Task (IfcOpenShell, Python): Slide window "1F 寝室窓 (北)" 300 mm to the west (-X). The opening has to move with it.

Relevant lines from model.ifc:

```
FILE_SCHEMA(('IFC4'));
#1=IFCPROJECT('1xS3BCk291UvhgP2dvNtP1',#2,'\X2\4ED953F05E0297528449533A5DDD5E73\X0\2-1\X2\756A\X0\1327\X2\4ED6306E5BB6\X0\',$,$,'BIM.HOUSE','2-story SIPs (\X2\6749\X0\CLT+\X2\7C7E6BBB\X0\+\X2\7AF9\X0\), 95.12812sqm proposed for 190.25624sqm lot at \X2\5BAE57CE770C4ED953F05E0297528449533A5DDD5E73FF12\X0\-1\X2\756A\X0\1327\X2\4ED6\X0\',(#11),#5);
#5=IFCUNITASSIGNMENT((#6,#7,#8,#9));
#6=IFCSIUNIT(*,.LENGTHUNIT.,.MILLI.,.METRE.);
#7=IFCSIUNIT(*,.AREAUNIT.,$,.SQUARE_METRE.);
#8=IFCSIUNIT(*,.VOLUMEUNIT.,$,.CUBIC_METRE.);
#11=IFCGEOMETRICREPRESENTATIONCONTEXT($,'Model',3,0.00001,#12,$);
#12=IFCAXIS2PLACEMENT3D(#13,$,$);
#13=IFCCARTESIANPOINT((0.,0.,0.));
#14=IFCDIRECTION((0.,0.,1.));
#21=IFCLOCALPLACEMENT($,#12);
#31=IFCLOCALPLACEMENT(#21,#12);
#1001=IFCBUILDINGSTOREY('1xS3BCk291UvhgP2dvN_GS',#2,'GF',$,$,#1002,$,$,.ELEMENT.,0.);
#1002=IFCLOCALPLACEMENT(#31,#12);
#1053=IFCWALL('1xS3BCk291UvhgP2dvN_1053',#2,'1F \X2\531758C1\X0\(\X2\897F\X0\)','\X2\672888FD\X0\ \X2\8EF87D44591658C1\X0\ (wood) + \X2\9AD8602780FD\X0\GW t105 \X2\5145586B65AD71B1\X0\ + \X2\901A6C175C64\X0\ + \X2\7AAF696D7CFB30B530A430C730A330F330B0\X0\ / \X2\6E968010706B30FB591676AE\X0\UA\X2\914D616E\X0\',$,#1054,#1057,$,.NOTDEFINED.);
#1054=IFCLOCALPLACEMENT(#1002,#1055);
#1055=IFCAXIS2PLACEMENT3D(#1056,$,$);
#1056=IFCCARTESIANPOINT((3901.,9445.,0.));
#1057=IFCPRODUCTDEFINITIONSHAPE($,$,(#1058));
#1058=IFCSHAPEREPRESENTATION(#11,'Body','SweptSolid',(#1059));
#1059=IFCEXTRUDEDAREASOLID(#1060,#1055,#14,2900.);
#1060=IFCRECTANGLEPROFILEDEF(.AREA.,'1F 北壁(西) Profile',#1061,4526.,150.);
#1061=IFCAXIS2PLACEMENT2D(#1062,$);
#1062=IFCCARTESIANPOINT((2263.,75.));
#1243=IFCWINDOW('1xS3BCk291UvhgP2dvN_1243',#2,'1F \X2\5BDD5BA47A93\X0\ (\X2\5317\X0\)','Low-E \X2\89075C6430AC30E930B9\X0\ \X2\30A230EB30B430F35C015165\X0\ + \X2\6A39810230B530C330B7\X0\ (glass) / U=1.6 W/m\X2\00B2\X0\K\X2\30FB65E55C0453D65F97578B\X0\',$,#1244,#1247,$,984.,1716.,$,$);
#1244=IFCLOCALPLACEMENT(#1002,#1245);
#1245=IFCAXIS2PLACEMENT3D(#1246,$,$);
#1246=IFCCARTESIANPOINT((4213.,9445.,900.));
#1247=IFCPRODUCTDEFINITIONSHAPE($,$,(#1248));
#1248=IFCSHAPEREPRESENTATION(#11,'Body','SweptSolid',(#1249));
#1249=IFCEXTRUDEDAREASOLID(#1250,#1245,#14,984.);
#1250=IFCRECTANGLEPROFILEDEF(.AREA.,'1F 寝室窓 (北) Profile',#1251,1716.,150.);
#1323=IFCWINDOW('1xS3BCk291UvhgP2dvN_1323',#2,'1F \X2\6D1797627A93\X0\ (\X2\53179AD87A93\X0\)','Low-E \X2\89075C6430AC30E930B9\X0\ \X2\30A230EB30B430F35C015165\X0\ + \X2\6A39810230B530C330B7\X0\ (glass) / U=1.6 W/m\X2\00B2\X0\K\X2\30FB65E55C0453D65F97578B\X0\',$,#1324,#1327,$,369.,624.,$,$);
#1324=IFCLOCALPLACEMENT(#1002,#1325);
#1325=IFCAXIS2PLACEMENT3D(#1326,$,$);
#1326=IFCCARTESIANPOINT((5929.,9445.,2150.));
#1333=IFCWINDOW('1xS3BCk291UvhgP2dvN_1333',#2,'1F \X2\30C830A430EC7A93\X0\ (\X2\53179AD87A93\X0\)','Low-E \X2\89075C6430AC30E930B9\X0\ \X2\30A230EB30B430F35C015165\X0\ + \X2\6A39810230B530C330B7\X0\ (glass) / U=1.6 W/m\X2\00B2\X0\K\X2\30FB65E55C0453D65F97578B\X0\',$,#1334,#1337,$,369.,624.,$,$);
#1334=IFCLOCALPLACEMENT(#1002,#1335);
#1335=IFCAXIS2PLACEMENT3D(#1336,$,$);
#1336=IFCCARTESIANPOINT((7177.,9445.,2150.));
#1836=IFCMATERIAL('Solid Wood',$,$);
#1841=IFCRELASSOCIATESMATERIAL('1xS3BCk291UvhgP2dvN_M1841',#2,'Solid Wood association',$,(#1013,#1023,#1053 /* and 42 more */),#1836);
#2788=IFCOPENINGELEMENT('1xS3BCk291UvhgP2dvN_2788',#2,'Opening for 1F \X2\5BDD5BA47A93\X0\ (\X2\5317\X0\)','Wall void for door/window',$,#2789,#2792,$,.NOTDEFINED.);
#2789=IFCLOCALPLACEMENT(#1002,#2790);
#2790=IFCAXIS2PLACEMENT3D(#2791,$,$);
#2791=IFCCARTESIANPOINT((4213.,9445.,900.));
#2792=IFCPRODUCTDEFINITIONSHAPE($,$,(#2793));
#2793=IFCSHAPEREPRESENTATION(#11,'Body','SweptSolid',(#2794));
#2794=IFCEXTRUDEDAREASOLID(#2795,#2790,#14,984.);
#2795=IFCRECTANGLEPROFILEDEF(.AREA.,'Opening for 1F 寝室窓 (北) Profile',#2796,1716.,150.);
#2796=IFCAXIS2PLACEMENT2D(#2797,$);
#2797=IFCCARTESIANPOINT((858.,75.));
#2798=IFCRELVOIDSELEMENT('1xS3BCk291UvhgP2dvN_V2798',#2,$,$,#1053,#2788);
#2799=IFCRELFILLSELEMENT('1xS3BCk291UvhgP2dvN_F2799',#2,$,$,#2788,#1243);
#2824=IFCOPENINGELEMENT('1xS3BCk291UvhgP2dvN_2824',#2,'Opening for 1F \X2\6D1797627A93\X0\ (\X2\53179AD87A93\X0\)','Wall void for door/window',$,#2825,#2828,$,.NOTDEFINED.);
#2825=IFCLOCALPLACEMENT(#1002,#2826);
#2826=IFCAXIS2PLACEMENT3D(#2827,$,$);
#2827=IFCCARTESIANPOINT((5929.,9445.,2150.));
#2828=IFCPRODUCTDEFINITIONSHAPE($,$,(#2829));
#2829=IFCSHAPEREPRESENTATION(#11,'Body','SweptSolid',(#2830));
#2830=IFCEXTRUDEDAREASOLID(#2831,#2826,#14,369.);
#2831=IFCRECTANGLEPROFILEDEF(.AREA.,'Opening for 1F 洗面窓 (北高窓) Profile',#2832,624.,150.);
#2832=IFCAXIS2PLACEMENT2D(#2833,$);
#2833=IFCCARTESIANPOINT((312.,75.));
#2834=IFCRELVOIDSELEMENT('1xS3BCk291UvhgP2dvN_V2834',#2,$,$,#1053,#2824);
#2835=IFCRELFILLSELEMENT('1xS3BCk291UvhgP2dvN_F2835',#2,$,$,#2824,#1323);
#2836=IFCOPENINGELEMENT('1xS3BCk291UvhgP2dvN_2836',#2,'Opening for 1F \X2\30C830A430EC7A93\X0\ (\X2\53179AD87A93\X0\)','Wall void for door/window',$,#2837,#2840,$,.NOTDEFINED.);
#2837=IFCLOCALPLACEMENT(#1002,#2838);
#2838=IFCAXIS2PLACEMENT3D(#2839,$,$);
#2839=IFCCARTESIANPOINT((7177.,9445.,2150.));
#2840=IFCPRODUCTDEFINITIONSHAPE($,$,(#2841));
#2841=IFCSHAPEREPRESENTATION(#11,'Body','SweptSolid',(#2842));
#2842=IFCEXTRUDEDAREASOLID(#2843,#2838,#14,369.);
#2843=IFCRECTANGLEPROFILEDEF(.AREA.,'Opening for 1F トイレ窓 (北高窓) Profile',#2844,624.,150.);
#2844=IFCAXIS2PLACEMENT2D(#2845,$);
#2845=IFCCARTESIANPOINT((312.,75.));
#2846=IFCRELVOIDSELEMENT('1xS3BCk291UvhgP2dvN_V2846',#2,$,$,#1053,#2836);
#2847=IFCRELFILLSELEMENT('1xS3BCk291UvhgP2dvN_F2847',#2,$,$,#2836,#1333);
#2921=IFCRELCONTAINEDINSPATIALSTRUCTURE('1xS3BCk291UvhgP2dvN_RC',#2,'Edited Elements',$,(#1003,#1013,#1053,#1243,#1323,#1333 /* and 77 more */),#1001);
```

```python
import ifcopenshell
import ifcopenshell.api.geometry
import ifcopenshell.util.placement
import ifcopenshell.util.unit

model = ifcopenshell.open("model.ifc")
unit_scale = ifcopenshell.util.unit.calculate_unit_scale(model)

window = model.by_guid("1xS3BCk291UvhgP2dvN_1243")
opening = window.FillsVoids[0].RelatingOpeningElement
wall = opening.VoidsElements[0].RelatingBuildingElement

wall_matrix = ifcopenshell.util.placement.get_local_placement(wall.ObjectPlacement)
shift = wall_matrix[:3, 0] * -0.3 / unit_scale
before = ifcopenshell.util.placement.get_local_placement(window.ObjectPlacement)[:3, 3].copy()

# The window is not placed relative to its opening, so move both.
for product in (opening, window):
    matrix = ifcopenshell.util.placement.get_local_placement(product.ObjectPlacement)
    matrix[:3, 3] += shift
    ifcopenshell.api.geometry.edit_object_placement(model, product=product, matrix=matrix, is_si=False)

after = ifcopenshell.util.placement.get_local_placement(window.ObjectPlacement)[:3, 3]
print("window moved by", (after - before).round(3) + 0.0)

model.write("model_edited.ifc")
```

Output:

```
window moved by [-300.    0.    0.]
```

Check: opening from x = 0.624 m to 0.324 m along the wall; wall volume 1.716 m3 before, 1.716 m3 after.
